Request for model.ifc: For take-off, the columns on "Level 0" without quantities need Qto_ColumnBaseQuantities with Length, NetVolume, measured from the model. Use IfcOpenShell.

First a look at what the model holds.

```python
import ifcopenshell
import ifcopenshell.util.element
import ifcopenshell.util.unit

model = ifcopenshell.open("model.ifc")
print(model.schema)
for unit_type in ("LENGTHUNIT", "AREAUNIT", "VOLUMEUNIT"):
    print(unit_type, ifcopenshell.util.unit.calculate_unit_scale(model, unit_type))
storey = next(s for s in model.by_type("IfcBuildingStorey") if s.Name == "Level 0")
columns = [e for e in ifcopenshell.util.element.get_decomposition(storey) if e.is_a("IfcColumn")]
for e in sorted(columns, key=lambda e: e.id()):
    print(e.id(), e.is_a(), e.Name, list(ifcopenshell.util.element.get_psets(e, qtos_only=True)), sep=" | ")
```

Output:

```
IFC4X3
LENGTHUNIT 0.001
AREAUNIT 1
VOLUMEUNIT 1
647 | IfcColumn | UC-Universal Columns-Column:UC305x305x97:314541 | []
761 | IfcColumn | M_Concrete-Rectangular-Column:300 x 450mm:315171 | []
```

```python
import ifcopenshell
import ifcopenshell.api.pset
import ifcopenshell.geom
import ifcopenshell.util.element
import ifcopenshell.util.shape
import ifcopenshell.util.unit

model = ifcopenshell.open("model.ifc")
unit_scale = ifcopenshell.util.unit.calculate_unit_scale(model)
volume_scale = ifcopenshell.util.unit.calculate_unit_scale(model, "VOLUMEUNIT")
settings = ifcopenshell.geom.settings()

storey = next(s for s in model.by_type("IfcBuildingStorey") if s.Name == "Level 0")
columns = [e for e in ifcopenshell.util.element.get_decomposition(storey) if e.is_a("IfcColumn")]

for e in sorted(columns, key=lambda e: e.id()):
    if ifcopenshell.util.element.get_psets(e, qtos_only=True, should_inherit=False):
        continue
    # Geometry comes back in metres, in the element's own axes.
    shape = ifcopenshell.geom.create_shape(settings, e)
    values = {
        "Length": ifcopenshell.util.shape.get_z(shape.geometry) / unit_scale,
        "NetVolume": ifcopenshell.util.shape.get_volume(shape.geometry) / volume_scale,
    }
    qto = ifcopenshell.api.pset.add_qto(model, product=e, name="Qto_ColumnBaseQuantities")
    ifcopenshell.api.pset.edit_qto(model, qto=qto, properties=values)
    print(e.id(), {k: round(v, 3) for k, v in values.items()})

model.write("model_updated.ifc")
```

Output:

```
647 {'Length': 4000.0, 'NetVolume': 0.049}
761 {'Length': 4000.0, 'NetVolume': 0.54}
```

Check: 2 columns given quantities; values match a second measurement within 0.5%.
